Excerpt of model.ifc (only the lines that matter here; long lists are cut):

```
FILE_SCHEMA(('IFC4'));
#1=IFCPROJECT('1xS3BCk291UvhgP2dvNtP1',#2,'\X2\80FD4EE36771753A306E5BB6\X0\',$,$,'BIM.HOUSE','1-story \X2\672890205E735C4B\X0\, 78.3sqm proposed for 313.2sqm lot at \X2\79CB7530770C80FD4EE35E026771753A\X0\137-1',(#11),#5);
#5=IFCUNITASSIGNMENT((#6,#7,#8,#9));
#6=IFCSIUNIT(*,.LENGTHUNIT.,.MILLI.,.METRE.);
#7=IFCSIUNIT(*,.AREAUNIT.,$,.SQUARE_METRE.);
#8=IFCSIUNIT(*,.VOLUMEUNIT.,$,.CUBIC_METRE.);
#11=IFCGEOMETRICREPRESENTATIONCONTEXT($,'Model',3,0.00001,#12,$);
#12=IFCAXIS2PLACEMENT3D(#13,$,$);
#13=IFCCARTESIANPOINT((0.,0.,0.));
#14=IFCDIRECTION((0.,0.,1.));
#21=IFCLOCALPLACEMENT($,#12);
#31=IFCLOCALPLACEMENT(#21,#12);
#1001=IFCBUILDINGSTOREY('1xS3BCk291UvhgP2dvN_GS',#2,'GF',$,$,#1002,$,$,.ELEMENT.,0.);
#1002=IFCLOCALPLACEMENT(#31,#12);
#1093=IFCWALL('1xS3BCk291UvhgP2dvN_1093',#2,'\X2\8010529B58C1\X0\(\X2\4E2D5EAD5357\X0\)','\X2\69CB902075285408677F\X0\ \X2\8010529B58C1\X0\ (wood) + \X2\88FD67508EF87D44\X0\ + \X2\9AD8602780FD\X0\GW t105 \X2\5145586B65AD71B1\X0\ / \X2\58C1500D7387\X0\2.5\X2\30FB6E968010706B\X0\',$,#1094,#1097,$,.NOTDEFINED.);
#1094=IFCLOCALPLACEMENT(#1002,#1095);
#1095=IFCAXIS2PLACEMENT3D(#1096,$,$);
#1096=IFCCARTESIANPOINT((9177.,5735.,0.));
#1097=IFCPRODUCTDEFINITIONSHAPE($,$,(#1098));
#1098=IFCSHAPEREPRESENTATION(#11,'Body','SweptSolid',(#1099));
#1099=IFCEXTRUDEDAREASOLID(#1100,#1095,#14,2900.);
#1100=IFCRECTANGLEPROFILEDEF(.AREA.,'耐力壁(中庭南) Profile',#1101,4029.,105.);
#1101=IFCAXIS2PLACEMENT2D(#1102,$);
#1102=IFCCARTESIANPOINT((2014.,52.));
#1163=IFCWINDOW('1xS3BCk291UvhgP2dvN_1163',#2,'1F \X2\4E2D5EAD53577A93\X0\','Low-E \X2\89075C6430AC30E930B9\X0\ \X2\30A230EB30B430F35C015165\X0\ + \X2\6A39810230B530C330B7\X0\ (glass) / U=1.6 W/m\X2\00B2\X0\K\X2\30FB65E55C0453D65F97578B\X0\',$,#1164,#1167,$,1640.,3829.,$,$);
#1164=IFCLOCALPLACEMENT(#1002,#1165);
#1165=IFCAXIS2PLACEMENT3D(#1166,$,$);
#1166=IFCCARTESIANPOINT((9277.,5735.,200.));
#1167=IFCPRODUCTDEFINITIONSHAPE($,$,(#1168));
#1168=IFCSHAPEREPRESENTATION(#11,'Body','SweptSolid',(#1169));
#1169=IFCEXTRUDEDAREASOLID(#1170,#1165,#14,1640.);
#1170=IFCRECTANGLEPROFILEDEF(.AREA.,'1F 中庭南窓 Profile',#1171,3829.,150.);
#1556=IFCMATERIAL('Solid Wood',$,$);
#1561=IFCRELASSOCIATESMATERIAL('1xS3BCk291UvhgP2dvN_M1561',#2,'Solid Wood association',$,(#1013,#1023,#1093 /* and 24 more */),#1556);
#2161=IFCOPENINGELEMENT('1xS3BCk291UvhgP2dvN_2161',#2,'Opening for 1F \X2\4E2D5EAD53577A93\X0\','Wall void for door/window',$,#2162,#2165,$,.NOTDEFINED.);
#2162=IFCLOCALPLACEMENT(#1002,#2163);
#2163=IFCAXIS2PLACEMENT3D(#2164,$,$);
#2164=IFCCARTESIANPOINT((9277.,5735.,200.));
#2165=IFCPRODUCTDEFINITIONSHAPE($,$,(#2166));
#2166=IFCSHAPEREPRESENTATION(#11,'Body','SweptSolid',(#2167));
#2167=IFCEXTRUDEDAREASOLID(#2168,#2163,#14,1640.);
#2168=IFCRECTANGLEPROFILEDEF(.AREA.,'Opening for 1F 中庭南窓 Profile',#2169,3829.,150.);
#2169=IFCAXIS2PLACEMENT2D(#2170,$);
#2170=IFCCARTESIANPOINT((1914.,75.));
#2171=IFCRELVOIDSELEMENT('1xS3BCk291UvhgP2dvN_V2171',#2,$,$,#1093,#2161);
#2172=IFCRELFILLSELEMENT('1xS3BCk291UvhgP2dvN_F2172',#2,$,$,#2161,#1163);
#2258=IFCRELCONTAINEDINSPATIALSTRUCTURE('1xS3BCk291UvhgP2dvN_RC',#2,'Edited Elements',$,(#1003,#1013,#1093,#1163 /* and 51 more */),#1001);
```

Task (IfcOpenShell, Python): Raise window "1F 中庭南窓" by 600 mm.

```python
import numpy as np
import ifcopenshell
import ifcopenshell.api.geometry
import ifcopenshell.util.placement
import ifcopenshell.util.unit

model = ifcopenshell.open("model.ifc")
unit_scale = ifcopenshell.util.unit.calculate_unit_scale(model)

window = model.by_guid("1xS3BCk291UvhgP2dvN_1163")
opening = window.FillsVoids[0].RelatingOpeningElement
dz = 0.6 / unit_scale

shift = np.array([0.0, 0.0, dz])
# The window is not placed relative to its opening, so move both.
for product in (opening, window):
    matrix = ifcopenshell.util.placement.get_local_placement(product.ObjectPlacement)
    matrix[:3, 3] += shift
    ifcopenshell.api.geometry.edit_object_placement(model, product=product, matrix=matrix, is_si=False)

print(f"moved by {dz * unit_scale:+.3f} m")

model.write("model-out.ifc")
```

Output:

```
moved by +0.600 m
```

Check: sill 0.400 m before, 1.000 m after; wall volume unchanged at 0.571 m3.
